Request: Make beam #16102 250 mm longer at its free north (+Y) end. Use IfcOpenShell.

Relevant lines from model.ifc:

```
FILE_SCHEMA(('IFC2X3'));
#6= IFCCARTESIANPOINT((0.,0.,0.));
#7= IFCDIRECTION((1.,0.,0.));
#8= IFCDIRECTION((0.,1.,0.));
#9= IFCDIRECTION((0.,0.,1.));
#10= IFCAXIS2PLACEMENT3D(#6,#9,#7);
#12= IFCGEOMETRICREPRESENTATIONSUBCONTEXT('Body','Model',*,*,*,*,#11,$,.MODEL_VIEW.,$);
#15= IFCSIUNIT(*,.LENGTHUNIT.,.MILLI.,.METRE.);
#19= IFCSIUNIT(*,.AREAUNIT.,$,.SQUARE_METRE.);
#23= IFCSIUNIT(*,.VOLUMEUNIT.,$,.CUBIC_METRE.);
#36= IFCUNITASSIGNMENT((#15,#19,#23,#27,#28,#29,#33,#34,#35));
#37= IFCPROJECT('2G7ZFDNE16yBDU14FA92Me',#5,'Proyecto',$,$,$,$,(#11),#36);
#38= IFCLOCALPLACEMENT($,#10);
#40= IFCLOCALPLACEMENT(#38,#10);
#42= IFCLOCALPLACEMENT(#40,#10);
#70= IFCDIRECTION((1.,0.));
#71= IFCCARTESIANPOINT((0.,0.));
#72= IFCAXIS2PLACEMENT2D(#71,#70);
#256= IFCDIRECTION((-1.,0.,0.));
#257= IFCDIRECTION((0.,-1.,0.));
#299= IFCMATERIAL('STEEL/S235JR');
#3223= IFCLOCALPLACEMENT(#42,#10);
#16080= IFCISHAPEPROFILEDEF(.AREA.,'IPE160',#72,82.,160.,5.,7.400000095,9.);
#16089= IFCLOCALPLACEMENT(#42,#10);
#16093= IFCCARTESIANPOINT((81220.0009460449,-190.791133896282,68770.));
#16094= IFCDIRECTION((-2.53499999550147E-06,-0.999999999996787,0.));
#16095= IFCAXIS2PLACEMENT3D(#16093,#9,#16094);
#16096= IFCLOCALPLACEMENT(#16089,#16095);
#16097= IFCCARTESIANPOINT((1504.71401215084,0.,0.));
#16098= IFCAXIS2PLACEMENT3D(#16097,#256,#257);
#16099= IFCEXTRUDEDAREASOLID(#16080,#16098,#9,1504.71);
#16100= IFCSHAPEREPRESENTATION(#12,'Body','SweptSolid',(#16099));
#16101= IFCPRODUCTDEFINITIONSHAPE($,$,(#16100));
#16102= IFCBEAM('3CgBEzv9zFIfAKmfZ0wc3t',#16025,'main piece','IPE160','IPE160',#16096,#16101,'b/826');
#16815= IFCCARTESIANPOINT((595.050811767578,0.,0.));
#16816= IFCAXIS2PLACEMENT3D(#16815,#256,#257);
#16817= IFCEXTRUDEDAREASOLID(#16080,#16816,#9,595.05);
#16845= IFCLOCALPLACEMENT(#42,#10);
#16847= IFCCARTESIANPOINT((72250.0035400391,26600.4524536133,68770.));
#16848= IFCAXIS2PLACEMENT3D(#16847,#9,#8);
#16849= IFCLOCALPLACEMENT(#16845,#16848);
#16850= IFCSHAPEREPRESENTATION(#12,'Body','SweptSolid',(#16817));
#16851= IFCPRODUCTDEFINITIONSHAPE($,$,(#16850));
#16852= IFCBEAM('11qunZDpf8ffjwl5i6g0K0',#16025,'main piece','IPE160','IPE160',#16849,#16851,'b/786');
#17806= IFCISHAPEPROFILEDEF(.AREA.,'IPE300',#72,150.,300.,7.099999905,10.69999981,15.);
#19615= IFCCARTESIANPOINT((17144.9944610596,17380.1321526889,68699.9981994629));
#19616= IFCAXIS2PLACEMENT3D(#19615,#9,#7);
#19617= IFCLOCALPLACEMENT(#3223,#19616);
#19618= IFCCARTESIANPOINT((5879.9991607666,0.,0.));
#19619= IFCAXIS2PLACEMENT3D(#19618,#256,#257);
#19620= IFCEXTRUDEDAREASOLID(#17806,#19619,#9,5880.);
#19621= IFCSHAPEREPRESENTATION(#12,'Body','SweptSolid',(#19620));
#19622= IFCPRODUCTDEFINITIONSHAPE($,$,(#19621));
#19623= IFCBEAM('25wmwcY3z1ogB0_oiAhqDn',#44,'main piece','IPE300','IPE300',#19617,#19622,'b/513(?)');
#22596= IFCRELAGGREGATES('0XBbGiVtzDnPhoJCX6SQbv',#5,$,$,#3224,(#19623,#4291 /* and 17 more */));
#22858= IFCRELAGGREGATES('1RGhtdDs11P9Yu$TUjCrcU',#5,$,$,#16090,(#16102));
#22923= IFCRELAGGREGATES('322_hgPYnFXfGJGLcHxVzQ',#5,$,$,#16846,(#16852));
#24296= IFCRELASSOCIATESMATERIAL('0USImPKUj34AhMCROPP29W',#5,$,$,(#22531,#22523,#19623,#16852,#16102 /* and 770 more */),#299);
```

```python
import ifcopenshell
import ifcopenshell.util.representation
import ifcopenshell.util.unit

model = ifcopenshell.open("model.ifc")
unit_scale = ifcopenshell.util.unit.calculate_unit_scale(model)

member = model.by_id(16102)
change = 0.25 / unit_scale

# The extrusion runs towards the end named, so only its depth changes.
body = ifcopenshell.util.representation.get_representation(member, "Model", "Body")
solid = body.Items[0]
old_length = solid.Depth
solid.Depth += change

print(f"length {old_length:g} -> {solid.Depth:g}")

model.write("model_v2.ifc")
```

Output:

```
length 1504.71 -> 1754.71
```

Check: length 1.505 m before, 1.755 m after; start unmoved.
